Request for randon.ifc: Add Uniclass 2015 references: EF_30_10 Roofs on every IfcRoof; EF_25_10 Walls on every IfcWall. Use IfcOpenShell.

First a look at what the model holds.

```python
import ifcopenshell

model = ifcopenshell.open("randon.ifc")
print(model.schema)
print("classifications:", [c.Name for c in model.by_type("IfcClassification")])
for ifc_class in ("IfcDoor", "IfcRoof", "IfcStair", "IfcWall", "IfcWindow"):
    print(ifc_class, len(model.by_type(ifc_class)))
```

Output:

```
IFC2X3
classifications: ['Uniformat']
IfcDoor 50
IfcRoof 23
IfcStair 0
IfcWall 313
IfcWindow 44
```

```python
import ifcopenshell
import ifcopenshell.api.classification

model = ifcopenshell.open("randon.ifc")

# IFC2X3 requires Source and Edition and has no link from the project to the system.
system = model.create_entity("IfcClassification", Source="NBS", Edition="2015", Name="Uniclass 2015")

codes = {
    "IfcRoof": ("EF_30_10", "Roofs"),
    "IfcWall": ("EF_25_10", "Walls"),
}
for ifc_class, (code, name) in codes.items():
    products = model.by_type(ifc_class)
    ifcopenshell.api.classification.add_reference(
        model, products=products, classification=system, identification=code, name=name
    )
    print(code, len(products))

model.write("randon_edited.ifc")
```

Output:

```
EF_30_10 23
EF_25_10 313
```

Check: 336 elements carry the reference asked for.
